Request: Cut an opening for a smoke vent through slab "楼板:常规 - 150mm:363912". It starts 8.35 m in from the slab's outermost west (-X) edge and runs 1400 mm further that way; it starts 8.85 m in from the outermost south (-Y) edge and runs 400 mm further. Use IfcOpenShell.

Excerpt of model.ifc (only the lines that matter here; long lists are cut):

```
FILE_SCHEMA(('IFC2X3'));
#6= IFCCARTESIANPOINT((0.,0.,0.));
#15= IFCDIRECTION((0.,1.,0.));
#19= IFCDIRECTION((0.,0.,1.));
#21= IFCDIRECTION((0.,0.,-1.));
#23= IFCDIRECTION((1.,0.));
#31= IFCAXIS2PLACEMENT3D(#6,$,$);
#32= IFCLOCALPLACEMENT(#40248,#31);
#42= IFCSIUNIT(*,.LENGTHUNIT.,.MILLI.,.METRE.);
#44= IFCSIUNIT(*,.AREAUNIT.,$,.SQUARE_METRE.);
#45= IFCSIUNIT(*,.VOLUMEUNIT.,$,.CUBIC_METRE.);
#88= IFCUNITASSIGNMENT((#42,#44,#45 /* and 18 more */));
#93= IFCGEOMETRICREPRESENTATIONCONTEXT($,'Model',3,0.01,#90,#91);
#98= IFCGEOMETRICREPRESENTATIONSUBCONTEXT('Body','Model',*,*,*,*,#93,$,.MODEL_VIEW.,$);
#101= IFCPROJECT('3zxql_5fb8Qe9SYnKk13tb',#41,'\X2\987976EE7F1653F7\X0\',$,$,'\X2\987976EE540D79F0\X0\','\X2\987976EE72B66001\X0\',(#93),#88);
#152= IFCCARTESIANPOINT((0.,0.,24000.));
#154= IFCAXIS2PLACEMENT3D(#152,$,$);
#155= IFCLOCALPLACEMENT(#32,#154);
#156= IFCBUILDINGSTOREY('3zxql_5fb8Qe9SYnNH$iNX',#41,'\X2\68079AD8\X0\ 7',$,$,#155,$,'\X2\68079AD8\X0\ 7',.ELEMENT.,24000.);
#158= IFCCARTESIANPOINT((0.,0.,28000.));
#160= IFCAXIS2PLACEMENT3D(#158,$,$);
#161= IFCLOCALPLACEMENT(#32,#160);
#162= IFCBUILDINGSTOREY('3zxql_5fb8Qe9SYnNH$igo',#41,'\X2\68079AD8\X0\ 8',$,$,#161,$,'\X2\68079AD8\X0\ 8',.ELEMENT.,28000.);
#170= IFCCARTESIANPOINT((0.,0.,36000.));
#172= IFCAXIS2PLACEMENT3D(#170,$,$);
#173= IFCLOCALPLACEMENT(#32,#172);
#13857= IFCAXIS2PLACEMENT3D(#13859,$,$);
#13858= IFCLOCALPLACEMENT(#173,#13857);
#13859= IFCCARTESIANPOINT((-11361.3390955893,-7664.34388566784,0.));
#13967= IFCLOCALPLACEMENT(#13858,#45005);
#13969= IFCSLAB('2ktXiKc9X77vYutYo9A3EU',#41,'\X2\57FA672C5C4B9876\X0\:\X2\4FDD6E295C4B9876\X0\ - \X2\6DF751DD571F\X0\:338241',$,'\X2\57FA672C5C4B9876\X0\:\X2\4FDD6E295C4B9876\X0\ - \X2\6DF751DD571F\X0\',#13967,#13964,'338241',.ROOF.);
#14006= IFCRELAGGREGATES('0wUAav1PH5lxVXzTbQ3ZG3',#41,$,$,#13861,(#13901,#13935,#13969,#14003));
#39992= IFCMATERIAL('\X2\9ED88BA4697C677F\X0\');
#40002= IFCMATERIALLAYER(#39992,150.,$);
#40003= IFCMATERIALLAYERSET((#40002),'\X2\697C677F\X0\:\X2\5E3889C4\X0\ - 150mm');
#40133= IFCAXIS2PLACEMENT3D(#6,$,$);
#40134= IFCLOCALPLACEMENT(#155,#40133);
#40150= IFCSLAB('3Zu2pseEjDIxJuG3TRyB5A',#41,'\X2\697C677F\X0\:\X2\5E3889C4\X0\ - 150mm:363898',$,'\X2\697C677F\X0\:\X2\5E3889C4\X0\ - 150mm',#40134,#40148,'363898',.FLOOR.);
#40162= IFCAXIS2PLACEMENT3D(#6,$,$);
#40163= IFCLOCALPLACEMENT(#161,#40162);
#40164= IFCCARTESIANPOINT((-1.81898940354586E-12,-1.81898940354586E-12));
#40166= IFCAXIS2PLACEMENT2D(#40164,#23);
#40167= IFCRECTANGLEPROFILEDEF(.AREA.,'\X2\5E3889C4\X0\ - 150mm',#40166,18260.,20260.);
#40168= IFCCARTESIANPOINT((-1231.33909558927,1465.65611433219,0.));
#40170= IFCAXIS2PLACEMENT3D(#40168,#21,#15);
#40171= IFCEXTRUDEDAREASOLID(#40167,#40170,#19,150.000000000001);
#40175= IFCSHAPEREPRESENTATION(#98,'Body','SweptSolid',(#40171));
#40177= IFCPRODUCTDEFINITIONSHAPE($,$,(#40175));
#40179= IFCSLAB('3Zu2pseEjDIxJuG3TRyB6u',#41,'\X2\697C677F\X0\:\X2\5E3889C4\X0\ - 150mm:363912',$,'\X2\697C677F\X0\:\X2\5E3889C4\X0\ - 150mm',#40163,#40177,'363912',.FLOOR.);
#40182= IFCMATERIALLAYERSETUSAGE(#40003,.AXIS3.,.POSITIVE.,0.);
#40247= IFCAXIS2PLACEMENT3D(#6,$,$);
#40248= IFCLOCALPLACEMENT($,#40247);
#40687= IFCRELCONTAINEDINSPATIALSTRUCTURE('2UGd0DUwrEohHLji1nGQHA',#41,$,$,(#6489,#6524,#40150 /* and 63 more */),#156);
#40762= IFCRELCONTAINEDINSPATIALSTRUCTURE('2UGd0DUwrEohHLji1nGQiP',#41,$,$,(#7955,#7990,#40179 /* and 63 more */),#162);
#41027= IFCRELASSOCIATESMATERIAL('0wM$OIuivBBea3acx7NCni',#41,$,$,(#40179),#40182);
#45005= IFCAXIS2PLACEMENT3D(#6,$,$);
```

```python
import numpy as np
import ifcopenshell
import ifcopenshell.api.feature
import ifcopenshell.api.geometry
import ifcopenshell.api.root
import ifcopenshell.geom
import ifcopenshell.util.placement
import ifcopenshell.util.representation
import ifcopenshell.util.shape
import ifcopenshell.util.unit

model = ifcopenshell.open("model.ifc")
unit_scale = ifcopenshell.util.unit.calculate_unit_scale(model)
settings = ifcopenshell.geom.settings()


def volume(element):
    """Net volume in cubic metres, openings subtracted."""
    shape = ifcopenshell.geom.create_shape(settings, element)
    return ifcopenshell.util.shape.get_volume(shape.geometry)


slab = model.by_guid("3Zu2pseEjDIxJuG3TRyB6u")
before = volume(slab)

# Extent in the slab's own axes, in metres. The edges named are its -X and -Y sides.
slab_shape = ifcopenshell.geom.create_shape(settings, slab)
vertices = ifcopenshell.util.shape.get_vertices(slab_shape.geometry)
x_min, y_min, bottom = vertices.min(axis=0)
top = vertices[:, 2].max()

opening = ifcopenshell.api.root.create_entity(model, ifc_class="IfcOpeningElement", name="Smoke vent opening")
context = ifcopenshell.util.representation.get_context(model, "Model", "Body", "MODEL_VIEW")
width, depth = 1.4, 0.4
outline = [(0.0, 0.0), (width, 0.0), (width, depth), (0.0, depth), (0.0, 0.0)]
# Overshoot both faces by 50 mm so the cut is clean.
shape = ifcopenshell.api.geometry.add_slab_representation(
    model, context=context, depth=top - bottom + 0.1, polyline=outline
)
ifcopenshell.api.geometry.assign_representation(model, product=opening, representation=shape)

matrix = ifcopenshell.util.placement.get_local_placement(slab.ObjectPlacement)
matrix[:, 3] = matrix @ np.append(np.array([x_min + 8.35, y_min + 8.85, bottom - 0.05]) / unit_scale, 1.0)
ifcopenshell.api.geometry.edit_object_placement(model, product=opening, matrix=matrix, is_si=False)
ifcopenshell.api.feature.add_feature(model, feature=opening, element=slab)

after = volume(slab)

print(f"slab volume {before:.3f} -> {after:.3f} m3")

model.write("model-out.ifc")
```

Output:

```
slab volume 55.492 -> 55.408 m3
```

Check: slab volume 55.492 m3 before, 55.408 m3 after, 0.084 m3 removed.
